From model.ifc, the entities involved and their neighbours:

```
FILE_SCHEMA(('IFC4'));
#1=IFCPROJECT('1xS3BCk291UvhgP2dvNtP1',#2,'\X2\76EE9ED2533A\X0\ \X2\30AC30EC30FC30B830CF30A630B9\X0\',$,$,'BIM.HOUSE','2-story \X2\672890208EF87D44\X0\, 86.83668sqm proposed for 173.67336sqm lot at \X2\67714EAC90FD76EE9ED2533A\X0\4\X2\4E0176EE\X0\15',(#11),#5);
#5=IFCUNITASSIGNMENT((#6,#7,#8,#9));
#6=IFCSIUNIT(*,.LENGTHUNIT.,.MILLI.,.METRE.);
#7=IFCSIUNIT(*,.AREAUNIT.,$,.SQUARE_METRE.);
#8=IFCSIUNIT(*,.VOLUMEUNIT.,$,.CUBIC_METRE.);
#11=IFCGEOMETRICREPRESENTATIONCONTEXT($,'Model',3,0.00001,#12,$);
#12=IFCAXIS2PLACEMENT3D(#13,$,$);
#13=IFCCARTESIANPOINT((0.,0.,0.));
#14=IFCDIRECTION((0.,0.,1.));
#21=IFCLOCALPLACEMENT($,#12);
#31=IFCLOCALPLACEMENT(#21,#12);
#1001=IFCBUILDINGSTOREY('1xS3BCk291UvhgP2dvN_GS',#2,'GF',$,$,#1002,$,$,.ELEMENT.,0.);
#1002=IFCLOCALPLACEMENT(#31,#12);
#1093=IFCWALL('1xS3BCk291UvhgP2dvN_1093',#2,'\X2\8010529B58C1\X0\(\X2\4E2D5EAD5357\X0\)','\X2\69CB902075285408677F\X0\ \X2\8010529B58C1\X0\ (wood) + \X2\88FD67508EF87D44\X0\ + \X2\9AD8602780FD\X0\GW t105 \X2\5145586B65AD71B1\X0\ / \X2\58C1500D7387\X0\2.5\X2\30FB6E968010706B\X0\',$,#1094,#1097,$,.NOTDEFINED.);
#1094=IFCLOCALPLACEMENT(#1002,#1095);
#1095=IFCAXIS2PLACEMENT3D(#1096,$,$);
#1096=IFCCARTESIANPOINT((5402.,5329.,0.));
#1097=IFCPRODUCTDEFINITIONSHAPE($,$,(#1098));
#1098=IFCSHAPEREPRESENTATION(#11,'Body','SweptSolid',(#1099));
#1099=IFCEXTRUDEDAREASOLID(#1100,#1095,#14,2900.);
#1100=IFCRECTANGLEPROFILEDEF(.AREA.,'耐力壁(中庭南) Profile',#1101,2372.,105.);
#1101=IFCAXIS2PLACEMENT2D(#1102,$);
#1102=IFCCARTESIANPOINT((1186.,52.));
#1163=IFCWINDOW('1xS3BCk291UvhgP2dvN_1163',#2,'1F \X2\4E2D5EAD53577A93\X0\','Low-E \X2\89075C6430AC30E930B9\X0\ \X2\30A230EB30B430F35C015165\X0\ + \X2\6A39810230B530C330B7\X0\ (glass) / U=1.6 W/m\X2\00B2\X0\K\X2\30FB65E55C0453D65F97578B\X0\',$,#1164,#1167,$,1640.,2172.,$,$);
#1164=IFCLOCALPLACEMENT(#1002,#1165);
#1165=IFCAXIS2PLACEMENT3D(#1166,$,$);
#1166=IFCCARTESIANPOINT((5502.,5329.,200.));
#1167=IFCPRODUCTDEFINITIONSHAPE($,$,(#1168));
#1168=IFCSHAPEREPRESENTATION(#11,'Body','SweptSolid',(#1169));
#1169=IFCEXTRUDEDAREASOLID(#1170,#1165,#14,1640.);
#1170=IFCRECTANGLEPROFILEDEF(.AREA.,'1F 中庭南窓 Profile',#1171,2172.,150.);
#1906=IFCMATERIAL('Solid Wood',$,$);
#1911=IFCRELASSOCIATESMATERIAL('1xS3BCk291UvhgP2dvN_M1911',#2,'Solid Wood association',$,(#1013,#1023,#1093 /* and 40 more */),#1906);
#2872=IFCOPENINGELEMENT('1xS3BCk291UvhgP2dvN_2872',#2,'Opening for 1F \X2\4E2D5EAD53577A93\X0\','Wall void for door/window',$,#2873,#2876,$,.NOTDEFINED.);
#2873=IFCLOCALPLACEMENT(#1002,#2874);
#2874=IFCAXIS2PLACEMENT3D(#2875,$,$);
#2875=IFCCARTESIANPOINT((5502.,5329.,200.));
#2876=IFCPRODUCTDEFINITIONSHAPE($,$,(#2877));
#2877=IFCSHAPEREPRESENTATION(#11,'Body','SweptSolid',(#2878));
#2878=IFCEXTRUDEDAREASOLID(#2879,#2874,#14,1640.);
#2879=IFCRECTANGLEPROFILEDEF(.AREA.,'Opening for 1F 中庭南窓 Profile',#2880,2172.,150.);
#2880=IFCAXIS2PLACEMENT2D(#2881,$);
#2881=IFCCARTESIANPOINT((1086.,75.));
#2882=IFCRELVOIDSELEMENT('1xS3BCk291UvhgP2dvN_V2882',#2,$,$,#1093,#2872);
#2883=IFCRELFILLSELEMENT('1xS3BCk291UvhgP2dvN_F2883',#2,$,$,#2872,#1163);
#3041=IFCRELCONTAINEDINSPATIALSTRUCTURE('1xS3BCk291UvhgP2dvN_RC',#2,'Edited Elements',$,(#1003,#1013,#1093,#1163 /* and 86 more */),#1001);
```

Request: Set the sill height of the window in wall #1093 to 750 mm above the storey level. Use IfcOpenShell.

```python
import numpy as np
import ifcopenshell
import ifcopenshell.api.geometry
import ifcopenshell.geom
import ifcopenshell.util.element
import ifcopenshell.util.placement
import ifcopenshell.util.shape
import ifcopenshell.util.unit

model = ifcopenshell.open("model.ifc")
unit_scale = ifcopenshell.util.unit.calculate_unit_scale(model)

window = model.by_guid("1xS3BCk291UvhgP2dvN_1163")
opening = window.FillsVoids[0].RelatingOpeningElement
storey = ifcopenshell.util.element.get_container(window, ifc_class="IfcBuildingStorey")
level = ifcopenshell.util.placement.get_local_placement(storey.ObjectPlacement)[2, 3]

# The opening's origin need not be at the sill, so measure its lowest point.
shape = ifcopenshell.geom.create_shape(ifcopenshell.geom.settings(), opening)
bottom = ifcopenshell.util.shape.get_shape_bottom_elevation(shape, shape.geometry) / unit_scale
dz = level + 0.75 / unit_scale - bottom

shift = np.array([0.0, 0.0, dz])
# The window is not placed relative to its opening, so move both.
for product in (opening, window):
    matrix = ifcopenshell.util.placement.get_local_placement(product.ObjectPlacement)
    matrix[:3, 3] += shift
    ifcopenshell.api.geometry.edit_object_placement(model, product=product, matrix=matrix, is_si=False)

print(f"moved by {dz * unit_scale:+.3f} m")

model.write("model_rev.ifc")
```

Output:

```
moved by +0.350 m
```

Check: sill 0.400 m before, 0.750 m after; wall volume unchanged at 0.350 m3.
